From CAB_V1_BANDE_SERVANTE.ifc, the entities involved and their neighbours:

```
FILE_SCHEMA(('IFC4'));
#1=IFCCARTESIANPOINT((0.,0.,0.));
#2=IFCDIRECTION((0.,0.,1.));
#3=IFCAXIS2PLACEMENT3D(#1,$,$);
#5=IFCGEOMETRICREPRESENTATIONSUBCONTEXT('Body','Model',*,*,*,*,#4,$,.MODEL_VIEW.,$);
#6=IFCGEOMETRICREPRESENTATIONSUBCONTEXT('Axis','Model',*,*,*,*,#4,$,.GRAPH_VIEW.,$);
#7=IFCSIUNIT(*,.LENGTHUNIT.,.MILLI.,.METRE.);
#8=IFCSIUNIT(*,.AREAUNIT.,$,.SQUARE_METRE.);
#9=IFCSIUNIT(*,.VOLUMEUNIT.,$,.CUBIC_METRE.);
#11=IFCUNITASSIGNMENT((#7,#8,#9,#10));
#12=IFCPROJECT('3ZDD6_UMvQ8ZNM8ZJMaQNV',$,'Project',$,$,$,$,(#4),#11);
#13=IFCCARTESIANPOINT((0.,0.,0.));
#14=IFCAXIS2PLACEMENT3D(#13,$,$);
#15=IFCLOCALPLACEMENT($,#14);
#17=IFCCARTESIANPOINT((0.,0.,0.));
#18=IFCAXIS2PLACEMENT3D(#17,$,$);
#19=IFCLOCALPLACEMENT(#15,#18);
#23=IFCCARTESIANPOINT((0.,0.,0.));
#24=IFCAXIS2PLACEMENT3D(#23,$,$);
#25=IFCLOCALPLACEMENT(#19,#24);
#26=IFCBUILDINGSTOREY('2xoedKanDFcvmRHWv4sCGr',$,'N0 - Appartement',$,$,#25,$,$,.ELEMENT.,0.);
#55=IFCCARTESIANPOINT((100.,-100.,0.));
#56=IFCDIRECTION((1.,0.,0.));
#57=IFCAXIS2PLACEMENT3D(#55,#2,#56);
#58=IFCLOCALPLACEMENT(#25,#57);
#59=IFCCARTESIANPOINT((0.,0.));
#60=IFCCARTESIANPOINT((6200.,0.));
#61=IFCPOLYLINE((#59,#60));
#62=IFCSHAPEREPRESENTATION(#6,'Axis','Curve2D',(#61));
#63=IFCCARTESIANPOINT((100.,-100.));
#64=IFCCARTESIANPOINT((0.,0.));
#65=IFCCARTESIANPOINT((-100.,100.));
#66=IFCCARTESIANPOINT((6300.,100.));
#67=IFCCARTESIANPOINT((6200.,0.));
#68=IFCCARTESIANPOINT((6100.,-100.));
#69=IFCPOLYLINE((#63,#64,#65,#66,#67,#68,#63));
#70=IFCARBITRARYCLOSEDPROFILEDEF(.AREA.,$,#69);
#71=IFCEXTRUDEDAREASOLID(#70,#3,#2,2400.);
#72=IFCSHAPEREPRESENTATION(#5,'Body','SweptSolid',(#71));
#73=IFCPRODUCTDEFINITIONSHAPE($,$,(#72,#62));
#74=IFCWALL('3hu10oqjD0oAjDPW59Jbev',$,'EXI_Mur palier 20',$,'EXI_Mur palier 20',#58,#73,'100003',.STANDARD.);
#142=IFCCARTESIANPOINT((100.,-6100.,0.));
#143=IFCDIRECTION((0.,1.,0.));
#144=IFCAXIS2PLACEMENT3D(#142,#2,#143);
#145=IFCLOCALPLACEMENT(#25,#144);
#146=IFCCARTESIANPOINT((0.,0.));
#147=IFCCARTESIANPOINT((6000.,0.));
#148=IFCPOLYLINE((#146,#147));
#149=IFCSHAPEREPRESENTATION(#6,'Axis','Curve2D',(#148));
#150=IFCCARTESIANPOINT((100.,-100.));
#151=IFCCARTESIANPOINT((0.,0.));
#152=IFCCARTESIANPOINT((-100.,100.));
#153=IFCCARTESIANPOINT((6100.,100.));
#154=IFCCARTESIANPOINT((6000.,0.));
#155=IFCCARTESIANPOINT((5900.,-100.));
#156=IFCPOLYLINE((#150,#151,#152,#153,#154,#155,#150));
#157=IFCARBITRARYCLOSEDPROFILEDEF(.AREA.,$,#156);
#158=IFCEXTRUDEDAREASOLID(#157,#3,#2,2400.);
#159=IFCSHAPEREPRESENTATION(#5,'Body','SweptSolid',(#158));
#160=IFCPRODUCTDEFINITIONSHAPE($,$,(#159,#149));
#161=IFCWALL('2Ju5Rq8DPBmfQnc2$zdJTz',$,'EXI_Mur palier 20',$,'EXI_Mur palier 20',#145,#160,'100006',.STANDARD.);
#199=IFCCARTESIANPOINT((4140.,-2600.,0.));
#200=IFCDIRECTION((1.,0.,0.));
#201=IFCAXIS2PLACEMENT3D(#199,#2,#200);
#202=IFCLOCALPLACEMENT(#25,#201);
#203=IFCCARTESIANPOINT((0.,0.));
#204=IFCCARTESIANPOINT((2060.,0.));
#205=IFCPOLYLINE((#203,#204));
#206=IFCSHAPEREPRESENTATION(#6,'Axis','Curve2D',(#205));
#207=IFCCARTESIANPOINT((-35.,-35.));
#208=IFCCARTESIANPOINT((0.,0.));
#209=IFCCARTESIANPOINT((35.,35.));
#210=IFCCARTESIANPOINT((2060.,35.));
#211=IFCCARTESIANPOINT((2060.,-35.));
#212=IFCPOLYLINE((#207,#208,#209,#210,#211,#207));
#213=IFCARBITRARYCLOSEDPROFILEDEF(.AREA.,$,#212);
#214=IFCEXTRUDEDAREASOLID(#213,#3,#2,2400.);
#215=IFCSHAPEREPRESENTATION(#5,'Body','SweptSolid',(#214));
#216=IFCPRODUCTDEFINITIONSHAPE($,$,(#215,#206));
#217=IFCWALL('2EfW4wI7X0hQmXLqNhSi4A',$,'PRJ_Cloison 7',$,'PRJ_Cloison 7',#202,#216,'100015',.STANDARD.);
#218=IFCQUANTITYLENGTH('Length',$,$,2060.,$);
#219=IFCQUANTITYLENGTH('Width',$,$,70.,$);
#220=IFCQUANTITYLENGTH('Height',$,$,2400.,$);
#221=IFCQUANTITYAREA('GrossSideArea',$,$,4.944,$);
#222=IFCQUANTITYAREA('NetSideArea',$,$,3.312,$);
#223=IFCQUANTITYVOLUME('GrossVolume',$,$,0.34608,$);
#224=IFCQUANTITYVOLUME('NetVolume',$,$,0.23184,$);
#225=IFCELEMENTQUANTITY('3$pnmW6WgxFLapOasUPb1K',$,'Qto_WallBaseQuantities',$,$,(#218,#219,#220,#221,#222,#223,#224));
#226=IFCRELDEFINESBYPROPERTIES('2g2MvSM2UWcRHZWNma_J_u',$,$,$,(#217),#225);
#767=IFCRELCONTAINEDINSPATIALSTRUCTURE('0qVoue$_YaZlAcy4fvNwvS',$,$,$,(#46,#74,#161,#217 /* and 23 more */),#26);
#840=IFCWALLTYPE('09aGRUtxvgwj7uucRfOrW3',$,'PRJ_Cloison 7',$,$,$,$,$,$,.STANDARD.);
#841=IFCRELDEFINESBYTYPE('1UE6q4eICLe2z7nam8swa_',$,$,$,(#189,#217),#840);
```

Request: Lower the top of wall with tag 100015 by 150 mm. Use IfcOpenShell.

```python
import ifcopenshell
import ifcopenshell.api.pset
import ifcopenshell.geom
import ifcopenshell.util.element
import ifcopenshell.util.representation
import ifcopenshell.util.shape
import ifcopenshell.util.unit

model = ifcopenshell.open("CAB_V1_BANDE_SERVANTE.ifc")
unit_scale = ifcopenshell.util.unit.calculate_unit_scale(model)
area_scale = ifcopenshell.util.unit.calculate_unit_scale(model, "AREAUNIT")
volume_scale = ifcopenshell.util.unit.calculate_unit_scale(model, "VOLUMEUNIT")
settings = ifcopenshell.geom.settings()


def volume(element):
    """Net volume in cubic metres, openings subtracted."""
    shape = ifcopenshell.geom.create_shape(settings, element)
    return ifcopenshell.util.shape.get_volume(shape.geometry)


wall = model.by_guid("2EfW4wI7X0hQmXLqNhSi4A")
before = volume(wall)

body = ifcopenshell.util.representation.get_representation(wall, "Model", "Body")
solid = body.Items[0]
old_height = solid.Depth
solid.Depth -= 0.15 / unit_scale
after = volume(wall)
thickness = 0.07  # wall thickness in metres

# Update the stored height, areas and volumes.
qto = model.by_id(ifcopenshell.util.element.get_pset(wall, "Qto_WallBaseQuantities", should_inherit=False)["id"])
ifcopenshell.api.pset.edit_qto(model, qto=qto, properties={
    "Height": solid.Depth,
    "GrossSideArea": ifcopenshell.util.element.get_pset(wall, "Qto_WallBaseQuantities", "GrossSideArea") * solid.Depth / old_height,
    "NetSideArea": after / thickness / area_scale,
    "GrossVolume": ifcopenshell.util.element.get_pset(wall, "Qto_WallBaseQuantities", "GrossVolume") * solid.Depth / old_height,
    "NetVolume": after / volume_scale,
})

print(f"height {old_height:g} -> {solid.Depth:g}, volume {before:.3f} -> {after:.3f} m3")

model.write("CAB_V1_BANDE_SERVANTE-out.ifc")
```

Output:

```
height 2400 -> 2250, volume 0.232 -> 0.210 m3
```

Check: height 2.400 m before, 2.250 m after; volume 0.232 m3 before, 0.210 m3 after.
